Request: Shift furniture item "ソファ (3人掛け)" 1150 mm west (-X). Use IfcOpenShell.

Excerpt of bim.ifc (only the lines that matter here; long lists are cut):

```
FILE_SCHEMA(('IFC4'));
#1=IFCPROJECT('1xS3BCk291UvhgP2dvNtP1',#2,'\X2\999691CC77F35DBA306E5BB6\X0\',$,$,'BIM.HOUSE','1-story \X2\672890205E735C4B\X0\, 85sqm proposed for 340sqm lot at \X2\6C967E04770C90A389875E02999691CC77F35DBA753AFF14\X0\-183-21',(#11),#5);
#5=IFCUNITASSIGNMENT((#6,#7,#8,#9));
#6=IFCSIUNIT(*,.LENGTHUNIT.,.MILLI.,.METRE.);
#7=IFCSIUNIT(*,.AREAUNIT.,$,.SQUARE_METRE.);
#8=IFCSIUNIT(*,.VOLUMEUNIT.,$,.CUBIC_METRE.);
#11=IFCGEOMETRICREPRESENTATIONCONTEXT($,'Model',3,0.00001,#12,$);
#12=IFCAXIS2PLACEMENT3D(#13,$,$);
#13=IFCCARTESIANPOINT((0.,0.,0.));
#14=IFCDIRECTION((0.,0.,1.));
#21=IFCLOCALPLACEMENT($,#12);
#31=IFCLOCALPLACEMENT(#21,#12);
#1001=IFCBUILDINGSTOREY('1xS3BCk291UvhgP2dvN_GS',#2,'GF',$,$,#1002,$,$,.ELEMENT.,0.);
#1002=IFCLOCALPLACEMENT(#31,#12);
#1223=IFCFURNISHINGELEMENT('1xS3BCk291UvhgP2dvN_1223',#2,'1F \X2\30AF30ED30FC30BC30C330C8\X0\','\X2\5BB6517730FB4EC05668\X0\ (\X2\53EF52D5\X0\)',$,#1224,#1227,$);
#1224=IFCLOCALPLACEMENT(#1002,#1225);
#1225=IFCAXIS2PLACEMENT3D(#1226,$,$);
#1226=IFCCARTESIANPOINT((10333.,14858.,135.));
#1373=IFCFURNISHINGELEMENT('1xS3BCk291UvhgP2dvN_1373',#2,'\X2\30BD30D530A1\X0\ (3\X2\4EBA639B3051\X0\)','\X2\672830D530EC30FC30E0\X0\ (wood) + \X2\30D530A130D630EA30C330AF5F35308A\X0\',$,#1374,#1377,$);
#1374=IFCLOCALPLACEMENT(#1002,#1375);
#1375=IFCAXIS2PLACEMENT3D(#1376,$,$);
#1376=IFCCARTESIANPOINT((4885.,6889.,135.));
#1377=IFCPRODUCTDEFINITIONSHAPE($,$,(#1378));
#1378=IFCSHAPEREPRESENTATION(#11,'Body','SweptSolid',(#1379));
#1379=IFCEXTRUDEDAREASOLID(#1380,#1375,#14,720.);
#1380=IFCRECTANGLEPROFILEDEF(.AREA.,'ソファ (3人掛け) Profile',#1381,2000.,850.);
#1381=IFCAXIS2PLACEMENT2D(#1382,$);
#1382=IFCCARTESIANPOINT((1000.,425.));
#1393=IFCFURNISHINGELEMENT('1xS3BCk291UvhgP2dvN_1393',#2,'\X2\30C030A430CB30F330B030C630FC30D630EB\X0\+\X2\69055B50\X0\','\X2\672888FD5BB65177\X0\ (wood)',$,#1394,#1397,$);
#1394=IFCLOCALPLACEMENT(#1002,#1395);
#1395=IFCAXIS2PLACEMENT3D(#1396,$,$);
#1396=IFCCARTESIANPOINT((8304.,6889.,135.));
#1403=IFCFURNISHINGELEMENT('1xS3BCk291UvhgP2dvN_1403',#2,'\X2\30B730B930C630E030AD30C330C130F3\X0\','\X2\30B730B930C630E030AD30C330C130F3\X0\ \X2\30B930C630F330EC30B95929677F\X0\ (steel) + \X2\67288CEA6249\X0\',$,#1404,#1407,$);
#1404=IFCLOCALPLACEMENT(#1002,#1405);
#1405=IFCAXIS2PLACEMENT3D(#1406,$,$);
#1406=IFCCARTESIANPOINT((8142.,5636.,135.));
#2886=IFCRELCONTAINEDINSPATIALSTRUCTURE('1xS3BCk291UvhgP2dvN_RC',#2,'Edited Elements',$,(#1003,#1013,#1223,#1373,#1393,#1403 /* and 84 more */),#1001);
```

```python
import ifcopenshell
import ifcopenshell.api.geometry
import ifcopenshell.util.placement
import ifcopenshell.util.unit

model = ifcopenshell.open("bim.ifc")
unit_scale = ifcopenshell.util.unit.calculate_unit_scale(model)

item = model.by_guid("1xS3BCk291UvhgP2dvN_1373")
matrix = ifcopenshell.util.placement.get_local_placement(item.ObjectPlacement)
matrix[0, 3] -= 1.15 / unit_scale
ifcopenshell.api.geometry.edit_object_placement(model, product=item, matrix=matrix, is_si=False)

print(ifcopenshell.util.placement.get_local_placement(item.ObjectPlacement).round(3) + 0.0)

model.write("bim-out.ifc")
```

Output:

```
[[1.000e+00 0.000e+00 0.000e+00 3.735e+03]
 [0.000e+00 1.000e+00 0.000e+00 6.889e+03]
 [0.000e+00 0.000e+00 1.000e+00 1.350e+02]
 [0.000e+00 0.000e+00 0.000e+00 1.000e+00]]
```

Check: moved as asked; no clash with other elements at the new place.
